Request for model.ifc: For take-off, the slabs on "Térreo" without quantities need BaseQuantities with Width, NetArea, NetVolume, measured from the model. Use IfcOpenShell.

First a look at what the model holds.

```python
import ifcopenshell
import ifcopenshell.util.element
import ifcopenshell.util.unit

model = ifcopenshell.open("model.ifc")
print(model.schema)
for unit_type in ("LENGTHUNIT", "AREAUNIT", "VOLUMEUNIT"):
    print(unit_type, ifcopenshell.util.unit.calculate_unit_scale(model, unit_type))
storey = next(s for s in model.by_type("IfcBuildingStorey") if s.Name == "Térreo")
slabs = [e for e in ifcopenshell.util.element.get_decomposition(storey) if e.is_a("IfcSlab")]
for e in sorted(slabs, key=lambda e: e.id()):
    print(e.id(), e.is_a(), e.Name, list(ifcopenshell.util.element.get_psets(e, qtos_only=True)), sep=" | ")
```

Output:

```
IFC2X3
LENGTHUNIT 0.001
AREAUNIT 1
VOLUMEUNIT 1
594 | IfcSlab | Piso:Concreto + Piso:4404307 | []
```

```python
import ifcopenshell
import ifcopenshell.api.pset
import ifcopenshell.geom
import ifcopenshell.util.element
import ifcopenshell.util.shape
import ifcopenshell.util.unit

model = ifcopenshell.open("model.ifc")
unit_scale = ifcopenshell.util.unit.calculate_unit_scale(model)
area_scale = ifcopenshell.util.unit.calculate_unit_scale(model, "AREAUNIT")
volume_scale = ifcopenshell.util.unit.calculate_unit_scale(model, "VOLUMEUNIT")
settings = ifcopenshell.geom.settings()

storey = next(s for s in model.by_type("IfcBuildingStorey") if s.Name == "Térreo")
slabs = [e for e in ifcopenshell.util.element.get_decomposition(storey) if e.is_a("IfcSlab")]

for e in sorted(slabs, key=lambda e: e.id()):
    if ifcopenshell.util.element.get_psets(e, qtos_only=True, should_inherit=False):
        continue
    # Geometry comes back in metres, in the element's own axes.
    shape = ifcopenshell.geom.create_shape(settings, e)
    values = {
        "Width": ifcopenshell.util.shape.get_z(shape.geometry) / unit_scale,
        "NetArea": ifcopenshell.util.shape.get_footprint_area(shape.geometry) / area_scale,
        "NetVolume": ifcopenshell.util.shape.get_volume(shape.geometry) / volume_scale,
    }
    qto = ifcopenshell.api.pset.add_qto(model, product=e, name="BaseQuantities")
    ifcopenshell.api.pset.edit_qto(model, qto=qto, properties=values)
    print(e.id(), {k: round(v, 3) for k, v in values.items()})

model.write("model_v2.ifc")
```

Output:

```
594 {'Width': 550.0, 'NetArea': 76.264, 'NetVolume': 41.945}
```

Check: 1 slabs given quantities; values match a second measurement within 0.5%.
